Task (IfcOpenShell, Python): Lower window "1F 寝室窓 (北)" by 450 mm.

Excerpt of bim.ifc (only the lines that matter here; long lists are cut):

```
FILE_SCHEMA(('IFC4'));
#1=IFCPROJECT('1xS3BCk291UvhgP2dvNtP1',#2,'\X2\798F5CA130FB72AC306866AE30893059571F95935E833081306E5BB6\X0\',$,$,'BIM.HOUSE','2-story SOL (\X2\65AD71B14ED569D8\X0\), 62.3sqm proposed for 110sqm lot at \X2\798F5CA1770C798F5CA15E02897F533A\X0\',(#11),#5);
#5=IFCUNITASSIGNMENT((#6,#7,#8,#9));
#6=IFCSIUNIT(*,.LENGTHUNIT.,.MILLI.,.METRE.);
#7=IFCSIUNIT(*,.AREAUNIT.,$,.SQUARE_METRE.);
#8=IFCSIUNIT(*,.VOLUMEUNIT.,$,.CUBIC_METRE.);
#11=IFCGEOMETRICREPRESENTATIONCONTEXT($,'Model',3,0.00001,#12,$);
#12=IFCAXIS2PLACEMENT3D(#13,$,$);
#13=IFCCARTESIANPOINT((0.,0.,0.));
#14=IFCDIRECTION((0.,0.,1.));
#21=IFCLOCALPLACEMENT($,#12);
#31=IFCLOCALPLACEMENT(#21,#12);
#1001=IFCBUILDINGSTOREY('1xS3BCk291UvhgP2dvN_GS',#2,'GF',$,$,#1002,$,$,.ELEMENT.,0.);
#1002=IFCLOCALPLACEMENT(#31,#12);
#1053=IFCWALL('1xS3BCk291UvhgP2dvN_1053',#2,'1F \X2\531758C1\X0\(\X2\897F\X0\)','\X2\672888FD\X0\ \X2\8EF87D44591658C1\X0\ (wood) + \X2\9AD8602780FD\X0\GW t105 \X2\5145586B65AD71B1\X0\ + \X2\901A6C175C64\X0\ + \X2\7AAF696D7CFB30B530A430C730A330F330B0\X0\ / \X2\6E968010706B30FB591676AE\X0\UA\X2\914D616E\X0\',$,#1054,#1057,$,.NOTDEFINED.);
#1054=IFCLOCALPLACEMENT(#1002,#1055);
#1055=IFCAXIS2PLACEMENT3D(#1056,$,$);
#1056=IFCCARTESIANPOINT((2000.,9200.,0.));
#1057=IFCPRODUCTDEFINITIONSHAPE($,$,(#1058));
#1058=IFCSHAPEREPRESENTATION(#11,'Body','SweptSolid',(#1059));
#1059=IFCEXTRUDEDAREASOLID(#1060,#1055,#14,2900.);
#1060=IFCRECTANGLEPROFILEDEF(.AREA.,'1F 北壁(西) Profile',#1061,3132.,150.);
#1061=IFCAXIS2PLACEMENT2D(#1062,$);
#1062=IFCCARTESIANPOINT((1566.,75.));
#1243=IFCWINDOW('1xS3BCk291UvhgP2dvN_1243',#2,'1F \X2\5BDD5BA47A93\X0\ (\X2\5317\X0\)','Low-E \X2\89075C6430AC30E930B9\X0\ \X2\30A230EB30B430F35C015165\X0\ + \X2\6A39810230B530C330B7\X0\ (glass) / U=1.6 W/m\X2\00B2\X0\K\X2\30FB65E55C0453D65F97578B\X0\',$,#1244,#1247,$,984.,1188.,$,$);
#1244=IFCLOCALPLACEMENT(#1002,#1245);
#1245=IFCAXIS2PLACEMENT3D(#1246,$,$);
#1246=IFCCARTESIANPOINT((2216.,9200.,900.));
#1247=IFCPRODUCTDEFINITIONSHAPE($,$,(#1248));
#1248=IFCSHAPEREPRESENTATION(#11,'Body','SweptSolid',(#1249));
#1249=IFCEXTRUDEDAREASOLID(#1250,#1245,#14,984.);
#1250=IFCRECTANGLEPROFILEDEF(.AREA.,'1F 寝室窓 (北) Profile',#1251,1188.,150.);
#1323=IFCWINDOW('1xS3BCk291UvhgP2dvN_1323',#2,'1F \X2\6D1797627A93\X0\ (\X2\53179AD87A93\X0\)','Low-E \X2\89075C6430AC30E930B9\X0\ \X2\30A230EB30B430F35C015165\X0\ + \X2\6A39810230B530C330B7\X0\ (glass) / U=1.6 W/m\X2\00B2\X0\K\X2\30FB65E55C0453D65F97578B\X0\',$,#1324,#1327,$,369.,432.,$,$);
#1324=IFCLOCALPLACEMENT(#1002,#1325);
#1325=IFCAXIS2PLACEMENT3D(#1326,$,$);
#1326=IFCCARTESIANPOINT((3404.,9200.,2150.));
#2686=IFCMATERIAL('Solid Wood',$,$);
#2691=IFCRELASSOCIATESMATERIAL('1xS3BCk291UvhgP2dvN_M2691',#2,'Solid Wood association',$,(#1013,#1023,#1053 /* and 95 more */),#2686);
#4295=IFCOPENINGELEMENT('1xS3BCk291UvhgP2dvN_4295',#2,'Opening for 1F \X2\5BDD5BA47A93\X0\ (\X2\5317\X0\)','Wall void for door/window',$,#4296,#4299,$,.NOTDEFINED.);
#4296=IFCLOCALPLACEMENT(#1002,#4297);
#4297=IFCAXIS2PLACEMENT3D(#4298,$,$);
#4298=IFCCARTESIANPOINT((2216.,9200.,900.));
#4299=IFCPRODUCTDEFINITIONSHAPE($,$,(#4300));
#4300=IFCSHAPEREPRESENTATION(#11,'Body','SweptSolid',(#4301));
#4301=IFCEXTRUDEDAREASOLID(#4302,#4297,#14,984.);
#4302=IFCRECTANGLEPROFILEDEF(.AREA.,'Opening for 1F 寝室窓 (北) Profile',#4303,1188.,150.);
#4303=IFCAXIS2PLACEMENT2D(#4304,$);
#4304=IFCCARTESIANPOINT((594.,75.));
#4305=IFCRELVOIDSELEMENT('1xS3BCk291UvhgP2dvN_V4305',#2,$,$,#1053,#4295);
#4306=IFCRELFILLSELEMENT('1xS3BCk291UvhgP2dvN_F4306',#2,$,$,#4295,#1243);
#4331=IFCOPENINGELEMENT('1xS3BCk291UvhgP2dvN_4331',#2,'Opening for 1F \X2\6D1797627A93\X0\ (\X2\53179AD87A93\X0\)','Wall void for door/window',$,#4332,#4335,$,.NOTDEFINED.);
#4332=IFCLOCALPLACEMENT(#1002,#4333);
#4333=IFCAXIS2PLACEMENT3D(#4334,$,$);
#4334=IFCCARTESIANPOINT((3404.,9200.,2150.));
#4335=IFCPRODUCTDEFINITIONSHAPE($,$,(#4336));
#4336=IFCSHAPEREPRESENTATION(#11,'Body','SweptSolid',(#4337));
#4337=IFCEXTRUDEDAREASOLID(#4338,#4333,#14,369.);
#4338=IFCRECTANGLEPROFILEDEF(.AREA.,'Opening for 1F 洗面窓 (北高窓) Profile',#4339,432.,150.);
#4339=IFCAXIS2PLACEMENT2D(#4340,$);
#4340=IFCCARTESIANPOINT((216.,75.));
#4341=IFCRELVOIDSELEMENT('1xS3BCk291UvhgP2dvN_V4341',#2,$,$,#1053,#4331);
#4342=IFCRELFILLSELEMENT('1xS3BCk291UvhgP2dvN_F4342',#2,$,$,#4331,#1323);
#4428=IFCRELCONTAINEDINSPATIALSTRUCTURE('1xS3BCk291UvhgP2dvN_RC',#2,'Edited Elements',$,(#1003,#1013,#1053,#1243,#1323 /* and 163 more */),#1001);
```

```python
import numpy as np
import ifcopenshell
import ifcopenshell.api.geometry
import ifcopenshell.util.placement
import ifcopenshell.util.unit

model = ifcopenshell.open("bim.ifc")
unit_scale = ifcopenshell.util.unit.calculate_unit_scale(model)

window = model.by_guid("1xS3BCk291UvhgP2dvN_1243")
opening = window.FillsVoids[0].RelatingOpeningElement
dz = -450.0

shift = np.array([0.0, 0.0, dz])
# The window is not placed relative to its opening, so move both.
for product in (opening, window):
    matrix = ifcopenshell.util.placement.get_local_placement(product.ObjectPlacement)
    matrix[:3, 3] += shift
    ifcopenshell.api.geometry.edit_object_placement(model, product=product, matrix=matrix, is_si=False)

print(f"moved by {dz * unit_scale:+.3f} m")

model.write("bim_updated.ifc")
```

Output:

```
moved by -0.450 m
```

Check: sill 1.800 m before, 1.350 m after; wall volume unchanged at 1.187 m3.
